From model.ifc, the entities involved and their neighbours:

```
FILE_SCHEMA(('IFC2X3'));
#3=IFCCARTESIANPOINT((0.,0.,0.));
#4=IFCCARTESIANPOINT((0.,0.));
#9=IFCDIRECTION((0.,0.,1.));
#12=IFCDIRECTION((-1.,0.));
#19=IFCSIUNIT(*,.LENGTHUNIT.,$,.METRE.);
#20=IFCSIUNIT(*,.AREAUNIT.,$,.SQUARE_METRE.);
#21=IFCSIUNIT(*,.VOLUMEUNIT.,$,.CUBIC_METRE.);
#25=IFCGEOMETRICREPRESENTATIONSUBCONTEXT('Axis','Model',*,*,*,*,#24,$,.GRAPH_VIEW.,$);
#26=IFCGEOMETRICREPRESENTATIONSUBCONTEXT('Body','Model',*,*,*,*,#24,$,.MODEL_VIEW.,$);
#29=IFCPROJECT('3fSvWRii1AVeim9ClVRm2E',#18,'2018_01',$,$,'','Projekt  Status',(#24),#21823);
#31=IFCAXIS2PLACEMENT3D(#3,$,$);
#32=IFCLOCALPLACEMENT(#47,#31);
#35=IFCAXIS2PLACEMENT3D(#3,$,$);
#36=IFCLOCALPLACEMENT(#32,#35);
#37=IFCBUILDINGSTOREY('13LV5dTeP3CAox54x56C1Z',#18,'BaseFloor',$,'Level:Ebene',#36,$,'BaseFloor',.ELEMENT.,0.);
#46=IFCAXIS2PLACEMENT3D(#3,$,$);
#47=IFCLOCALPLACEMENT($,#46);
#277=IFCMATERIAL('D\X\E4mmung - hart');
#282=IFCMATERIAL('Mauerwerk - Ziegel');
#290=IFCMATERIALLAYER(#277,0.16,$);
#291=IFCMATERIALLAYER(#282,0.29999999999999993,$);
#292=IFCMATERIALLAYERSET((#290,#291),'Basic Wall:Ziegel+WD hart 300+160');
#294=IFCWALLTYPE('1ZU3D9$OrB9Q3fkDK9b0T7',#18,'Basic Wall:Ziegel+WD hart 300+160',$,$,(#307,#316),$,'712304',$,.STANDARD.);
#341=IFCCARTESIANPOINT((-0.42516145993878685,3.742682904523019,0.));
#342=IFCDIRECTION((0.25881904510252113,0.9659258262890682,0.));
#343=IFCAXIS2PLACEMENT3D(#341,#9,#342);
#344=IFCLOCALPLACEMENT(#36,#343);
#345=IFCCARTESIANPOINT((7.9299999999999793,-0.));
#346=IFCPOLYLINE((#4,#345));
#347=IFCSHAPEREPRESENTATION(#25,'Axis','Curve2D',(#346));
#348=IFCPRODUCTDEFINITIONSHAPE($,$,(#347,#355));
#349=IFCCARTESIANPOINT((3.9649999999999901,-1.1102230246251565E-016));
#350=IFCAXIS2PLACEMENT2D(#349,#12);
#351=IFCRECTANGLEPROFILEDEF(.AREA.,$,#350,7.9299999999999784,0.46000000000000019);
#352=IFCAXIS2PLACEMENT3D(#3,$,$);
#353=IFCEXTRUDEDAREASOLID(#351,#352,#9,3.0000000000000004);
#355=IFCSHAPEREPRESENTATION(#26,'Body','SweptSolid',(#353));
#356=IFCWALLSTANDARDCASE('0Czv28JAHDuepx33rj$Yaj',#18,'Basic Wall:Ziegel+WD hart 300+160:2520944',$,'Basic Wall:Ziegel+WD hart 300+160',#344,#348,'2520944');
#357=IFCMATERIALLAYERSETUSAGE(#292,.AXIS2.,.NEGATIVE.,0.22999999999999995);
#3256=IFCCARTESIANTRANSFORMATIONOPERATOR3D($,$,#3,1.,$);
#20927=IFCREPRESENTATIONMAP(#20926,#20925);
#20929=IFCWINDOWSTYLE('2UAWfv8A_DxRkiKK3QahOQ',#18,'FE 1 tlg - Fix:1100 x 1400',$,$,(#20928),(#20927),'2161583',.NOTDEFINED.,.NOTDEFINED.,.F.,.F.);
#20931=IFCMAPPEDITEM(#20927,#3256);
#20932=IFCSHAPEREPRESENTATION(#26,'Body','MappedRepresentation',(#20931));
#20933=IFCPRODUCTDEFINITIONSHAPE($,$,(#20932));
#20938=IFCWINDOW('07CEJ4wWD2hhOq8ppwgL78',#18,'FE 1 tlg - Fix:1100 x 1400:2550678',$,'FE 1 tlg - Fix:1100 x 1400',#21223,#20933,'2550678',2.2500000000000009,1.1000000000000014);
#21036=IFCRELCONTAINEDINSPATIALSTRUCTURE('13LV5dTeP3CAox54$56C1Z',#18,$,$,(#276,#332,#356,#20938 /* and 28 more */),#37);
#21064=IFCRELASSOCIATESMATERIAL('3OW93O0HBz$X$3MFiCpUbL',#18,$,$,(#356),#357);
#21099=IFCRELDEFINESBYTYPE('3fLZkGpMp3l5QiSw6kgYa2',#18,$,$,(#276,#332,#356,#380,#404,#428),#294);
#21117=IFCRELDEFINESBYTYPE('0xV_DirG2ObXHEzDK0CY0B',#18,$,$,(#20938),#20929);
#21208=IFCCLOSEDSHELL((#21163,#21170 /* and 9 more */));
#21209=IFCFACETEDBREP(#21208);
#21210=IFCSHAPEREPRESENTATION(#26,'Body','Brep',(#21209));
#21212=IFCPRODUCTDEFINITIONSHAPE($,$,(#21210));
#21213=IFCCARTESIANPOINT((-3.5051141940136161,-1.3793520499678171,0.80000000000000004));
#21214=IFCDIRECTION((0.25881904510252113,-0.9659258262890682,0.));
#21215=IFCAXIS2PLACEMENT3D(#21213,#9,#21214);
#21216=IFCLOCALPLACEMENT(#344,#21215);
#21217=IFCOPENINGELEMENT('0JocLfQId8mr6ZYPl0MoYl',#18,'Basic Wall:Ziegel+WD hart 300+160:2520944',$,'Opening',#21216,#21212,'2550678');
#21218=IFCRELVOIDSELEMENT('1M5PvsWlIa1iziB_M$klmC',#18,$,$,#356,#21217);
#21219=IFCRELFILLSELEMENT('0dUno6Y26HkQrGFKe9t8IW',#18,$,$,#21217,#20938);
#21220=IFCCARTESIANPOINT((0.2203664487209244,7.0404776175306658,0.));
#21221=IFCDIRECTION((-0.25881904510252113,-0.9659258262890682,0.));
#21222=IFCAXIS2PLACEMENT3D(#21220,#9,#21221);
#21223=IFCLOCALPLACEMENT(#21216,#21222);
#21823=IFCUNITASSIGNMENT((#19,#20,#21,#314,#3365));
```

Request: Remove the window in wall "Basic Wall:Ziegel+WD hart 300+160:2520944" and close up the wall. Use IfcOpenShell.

```python
import ifcopenshell
import ifcopenshell.api.feature
import ifcopenshell.api.root
import ifcopenshell.geom
import ifcopenshell.util.shape

model = ifcopenshell.open("model.ifc")
settings = ifcopenshell.geom.settings()


def volume(element):
    """Net volume in cubic metres, openings subtracted."""
    shape = ifcopenshell.geom.create_shape(settings, element)
    return ifcopenshell.util.shape.get_volume(shape.geometry)


window = model.by_id(20938)
opening = window.FillsVoids[0].RelatingOpeningElement
wall = opening.VoidsElements[0].RelatingBuildingElement
before = volume(wall)

ifcopenshell.api.root.remove_product(model, product=window)
ifcopenshell.api.feature.remove_feature(model, feature=opening)

after = volume(wall)

print(f"wall volume {before:.3f} -> {after:.3f} m3")

model.write("model_edited.ifc")
```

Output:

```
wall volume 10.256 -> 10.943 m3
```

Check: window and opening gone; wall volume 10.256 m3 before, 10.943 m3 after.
